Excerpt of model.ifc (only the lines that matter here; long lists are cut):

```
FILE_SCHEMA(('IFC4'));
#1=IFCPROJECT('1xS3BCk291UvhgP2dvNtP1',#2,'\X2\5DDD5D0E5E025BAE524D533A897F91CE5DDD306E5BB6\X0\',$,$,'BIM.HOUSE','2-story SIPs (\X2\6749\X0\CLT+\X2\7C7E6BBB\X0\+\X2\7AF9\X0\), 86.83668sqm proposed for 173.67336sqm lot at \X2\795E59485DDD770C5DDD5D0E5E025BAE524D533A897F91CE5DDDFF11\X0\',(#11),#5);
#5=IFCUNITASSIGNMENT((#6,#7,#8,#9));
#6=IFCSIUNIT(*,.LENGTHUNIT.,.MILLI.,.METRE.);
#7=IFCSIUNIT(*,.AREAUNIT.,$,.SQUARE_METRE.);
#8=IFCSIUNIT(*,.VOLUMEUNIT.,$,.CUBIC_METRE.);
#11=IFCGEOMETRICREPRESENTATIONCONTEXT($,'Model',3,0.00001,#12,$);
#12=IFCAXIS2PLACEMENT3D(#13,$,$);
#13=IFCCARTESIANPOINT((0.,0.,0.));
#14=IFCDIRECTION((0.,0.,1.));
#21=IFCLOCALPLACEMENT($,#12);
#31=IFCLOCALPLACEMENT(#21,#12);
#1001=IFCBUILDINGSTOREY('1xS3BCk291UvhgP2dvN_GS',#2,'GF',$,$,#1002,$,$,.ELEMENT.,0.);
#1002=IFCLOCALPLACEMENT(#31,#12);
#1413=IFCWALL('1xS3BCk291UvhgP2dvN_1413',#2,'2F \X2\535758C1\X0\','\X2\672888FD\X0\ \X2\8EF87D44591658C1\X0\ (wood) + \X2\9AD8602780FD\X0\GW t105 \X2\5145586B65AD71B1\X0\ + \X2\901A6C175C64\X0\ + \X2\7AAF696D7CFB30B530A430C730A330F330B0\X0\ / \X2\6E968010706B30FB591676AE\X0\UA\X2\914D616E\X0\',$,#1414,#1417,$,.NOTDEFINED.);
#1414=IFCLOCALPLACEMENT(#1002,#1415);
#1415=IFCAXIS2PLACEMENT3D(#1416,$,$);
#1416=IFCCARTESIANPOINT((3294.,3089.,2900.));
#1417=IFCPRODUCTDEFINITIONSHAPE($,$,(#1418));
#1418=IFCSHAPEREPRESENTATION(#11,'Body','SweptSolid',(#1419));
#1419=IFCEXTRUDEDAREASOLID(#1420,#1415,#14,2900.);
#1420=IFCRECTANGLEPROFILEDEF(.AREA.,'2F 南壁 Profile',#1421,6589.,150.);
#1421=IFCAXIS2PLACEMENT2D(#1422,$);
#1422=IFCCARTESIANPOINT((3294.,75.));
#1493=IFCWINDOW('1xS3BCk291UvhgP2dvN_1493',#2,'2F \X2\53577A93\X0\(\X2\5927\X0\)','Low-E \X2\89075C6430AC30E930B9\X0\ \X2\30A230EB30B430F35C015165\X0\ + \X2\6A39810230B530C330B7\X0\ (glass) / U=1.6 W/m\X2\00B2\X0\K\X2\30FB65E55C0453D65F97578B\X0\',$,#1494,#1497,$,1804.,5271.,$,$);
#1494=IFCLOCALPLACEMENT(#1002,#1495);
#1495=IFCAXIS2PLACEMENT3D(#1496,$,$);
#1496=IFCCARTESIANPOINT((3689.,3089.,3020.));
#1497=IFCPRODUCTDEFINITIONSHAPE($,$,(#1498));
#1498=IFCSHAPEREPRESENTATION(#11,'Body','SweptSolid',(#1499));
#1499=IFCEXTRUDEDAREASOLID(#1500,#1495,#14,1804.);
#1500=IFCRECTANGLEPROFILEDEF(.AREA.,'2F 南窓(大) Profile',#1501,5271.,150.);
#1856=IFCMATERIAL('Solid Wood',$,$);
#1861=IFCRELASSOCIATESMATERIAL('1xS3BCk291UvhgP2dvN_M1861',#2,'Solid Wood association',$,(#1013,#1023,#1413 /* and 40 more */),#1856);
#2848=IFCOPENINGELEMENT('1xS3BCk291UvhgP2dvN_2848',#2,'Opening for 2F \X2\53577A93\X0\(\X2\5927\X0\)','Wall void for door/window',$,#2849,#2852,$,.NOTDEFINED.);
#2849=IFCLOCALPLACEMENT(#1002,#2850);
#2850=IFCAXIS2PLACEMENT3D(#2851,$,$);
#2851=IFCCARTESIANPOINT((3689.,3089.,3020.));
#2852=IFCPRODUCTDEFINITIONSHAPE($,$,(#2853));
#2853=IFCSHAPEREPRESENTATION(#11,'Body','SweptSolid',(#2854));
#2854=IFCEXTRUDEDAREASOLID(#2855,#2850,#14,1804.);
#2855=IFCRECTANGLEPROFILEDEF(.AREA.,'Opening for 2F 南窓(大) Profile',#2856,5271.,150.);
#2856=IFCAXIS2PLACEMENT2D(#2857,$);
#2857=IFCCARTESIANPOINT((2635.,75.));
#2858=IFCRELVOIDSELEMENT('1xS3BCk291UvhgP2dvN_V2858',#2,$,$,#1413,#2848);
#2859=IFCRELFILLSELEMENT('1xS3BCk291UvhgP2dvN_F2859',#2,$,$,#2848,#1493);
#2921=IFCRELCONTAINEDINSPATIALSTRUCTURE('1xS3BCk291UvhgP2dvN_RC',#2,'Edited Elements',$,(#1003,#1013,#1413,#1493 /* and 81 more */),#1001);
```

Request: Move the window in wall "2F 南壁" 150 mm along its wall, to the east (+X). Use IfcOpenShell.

```python
import ifcopenshell
import ifcopenshell.api.geometry
import ifcopenshell.util.placement

model = ifcopenshell.open("model.ifc")

window = model.by_guid("1xS3BCk291UvhgP2dvN_1493")
opening = window.FillsVoids[0].RelatingOpeningElement
wall = opening.VoidsElements[0].RelatingBuildingElement

wall_matrix = ifcopenshell.util.placement.get_local_placement(wall.ObjectPlacement)
shift = wall_matrix[:3, 0] * 150.0
before = ifcopenshell.util.placement.get_local_placement(window.ObjectPlacement)[:3, 3].copy()

# The window is not placed relative to its opening, so move both.
for product in (opening, window):
    matrix = ifcopenshell.util.placement.get_local_placement(product.ObjectPlacement)
    matrix[:3, 3] += shift
    ifcopenshell.api.geometry.edit_object_placement(model, product=product, matrix=matrix, is_si=False)

after = ifcopenshell.util.placement.get_local_placement(window.ObjectPlacement)[:3, 3]
print("window moved by", (after - before).round(3) + 0.0)

model.write("model_v2.ifc")
```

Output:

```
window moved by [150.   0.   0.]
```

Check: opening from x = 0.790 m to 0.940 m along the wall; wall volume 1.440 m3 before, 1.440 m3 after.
